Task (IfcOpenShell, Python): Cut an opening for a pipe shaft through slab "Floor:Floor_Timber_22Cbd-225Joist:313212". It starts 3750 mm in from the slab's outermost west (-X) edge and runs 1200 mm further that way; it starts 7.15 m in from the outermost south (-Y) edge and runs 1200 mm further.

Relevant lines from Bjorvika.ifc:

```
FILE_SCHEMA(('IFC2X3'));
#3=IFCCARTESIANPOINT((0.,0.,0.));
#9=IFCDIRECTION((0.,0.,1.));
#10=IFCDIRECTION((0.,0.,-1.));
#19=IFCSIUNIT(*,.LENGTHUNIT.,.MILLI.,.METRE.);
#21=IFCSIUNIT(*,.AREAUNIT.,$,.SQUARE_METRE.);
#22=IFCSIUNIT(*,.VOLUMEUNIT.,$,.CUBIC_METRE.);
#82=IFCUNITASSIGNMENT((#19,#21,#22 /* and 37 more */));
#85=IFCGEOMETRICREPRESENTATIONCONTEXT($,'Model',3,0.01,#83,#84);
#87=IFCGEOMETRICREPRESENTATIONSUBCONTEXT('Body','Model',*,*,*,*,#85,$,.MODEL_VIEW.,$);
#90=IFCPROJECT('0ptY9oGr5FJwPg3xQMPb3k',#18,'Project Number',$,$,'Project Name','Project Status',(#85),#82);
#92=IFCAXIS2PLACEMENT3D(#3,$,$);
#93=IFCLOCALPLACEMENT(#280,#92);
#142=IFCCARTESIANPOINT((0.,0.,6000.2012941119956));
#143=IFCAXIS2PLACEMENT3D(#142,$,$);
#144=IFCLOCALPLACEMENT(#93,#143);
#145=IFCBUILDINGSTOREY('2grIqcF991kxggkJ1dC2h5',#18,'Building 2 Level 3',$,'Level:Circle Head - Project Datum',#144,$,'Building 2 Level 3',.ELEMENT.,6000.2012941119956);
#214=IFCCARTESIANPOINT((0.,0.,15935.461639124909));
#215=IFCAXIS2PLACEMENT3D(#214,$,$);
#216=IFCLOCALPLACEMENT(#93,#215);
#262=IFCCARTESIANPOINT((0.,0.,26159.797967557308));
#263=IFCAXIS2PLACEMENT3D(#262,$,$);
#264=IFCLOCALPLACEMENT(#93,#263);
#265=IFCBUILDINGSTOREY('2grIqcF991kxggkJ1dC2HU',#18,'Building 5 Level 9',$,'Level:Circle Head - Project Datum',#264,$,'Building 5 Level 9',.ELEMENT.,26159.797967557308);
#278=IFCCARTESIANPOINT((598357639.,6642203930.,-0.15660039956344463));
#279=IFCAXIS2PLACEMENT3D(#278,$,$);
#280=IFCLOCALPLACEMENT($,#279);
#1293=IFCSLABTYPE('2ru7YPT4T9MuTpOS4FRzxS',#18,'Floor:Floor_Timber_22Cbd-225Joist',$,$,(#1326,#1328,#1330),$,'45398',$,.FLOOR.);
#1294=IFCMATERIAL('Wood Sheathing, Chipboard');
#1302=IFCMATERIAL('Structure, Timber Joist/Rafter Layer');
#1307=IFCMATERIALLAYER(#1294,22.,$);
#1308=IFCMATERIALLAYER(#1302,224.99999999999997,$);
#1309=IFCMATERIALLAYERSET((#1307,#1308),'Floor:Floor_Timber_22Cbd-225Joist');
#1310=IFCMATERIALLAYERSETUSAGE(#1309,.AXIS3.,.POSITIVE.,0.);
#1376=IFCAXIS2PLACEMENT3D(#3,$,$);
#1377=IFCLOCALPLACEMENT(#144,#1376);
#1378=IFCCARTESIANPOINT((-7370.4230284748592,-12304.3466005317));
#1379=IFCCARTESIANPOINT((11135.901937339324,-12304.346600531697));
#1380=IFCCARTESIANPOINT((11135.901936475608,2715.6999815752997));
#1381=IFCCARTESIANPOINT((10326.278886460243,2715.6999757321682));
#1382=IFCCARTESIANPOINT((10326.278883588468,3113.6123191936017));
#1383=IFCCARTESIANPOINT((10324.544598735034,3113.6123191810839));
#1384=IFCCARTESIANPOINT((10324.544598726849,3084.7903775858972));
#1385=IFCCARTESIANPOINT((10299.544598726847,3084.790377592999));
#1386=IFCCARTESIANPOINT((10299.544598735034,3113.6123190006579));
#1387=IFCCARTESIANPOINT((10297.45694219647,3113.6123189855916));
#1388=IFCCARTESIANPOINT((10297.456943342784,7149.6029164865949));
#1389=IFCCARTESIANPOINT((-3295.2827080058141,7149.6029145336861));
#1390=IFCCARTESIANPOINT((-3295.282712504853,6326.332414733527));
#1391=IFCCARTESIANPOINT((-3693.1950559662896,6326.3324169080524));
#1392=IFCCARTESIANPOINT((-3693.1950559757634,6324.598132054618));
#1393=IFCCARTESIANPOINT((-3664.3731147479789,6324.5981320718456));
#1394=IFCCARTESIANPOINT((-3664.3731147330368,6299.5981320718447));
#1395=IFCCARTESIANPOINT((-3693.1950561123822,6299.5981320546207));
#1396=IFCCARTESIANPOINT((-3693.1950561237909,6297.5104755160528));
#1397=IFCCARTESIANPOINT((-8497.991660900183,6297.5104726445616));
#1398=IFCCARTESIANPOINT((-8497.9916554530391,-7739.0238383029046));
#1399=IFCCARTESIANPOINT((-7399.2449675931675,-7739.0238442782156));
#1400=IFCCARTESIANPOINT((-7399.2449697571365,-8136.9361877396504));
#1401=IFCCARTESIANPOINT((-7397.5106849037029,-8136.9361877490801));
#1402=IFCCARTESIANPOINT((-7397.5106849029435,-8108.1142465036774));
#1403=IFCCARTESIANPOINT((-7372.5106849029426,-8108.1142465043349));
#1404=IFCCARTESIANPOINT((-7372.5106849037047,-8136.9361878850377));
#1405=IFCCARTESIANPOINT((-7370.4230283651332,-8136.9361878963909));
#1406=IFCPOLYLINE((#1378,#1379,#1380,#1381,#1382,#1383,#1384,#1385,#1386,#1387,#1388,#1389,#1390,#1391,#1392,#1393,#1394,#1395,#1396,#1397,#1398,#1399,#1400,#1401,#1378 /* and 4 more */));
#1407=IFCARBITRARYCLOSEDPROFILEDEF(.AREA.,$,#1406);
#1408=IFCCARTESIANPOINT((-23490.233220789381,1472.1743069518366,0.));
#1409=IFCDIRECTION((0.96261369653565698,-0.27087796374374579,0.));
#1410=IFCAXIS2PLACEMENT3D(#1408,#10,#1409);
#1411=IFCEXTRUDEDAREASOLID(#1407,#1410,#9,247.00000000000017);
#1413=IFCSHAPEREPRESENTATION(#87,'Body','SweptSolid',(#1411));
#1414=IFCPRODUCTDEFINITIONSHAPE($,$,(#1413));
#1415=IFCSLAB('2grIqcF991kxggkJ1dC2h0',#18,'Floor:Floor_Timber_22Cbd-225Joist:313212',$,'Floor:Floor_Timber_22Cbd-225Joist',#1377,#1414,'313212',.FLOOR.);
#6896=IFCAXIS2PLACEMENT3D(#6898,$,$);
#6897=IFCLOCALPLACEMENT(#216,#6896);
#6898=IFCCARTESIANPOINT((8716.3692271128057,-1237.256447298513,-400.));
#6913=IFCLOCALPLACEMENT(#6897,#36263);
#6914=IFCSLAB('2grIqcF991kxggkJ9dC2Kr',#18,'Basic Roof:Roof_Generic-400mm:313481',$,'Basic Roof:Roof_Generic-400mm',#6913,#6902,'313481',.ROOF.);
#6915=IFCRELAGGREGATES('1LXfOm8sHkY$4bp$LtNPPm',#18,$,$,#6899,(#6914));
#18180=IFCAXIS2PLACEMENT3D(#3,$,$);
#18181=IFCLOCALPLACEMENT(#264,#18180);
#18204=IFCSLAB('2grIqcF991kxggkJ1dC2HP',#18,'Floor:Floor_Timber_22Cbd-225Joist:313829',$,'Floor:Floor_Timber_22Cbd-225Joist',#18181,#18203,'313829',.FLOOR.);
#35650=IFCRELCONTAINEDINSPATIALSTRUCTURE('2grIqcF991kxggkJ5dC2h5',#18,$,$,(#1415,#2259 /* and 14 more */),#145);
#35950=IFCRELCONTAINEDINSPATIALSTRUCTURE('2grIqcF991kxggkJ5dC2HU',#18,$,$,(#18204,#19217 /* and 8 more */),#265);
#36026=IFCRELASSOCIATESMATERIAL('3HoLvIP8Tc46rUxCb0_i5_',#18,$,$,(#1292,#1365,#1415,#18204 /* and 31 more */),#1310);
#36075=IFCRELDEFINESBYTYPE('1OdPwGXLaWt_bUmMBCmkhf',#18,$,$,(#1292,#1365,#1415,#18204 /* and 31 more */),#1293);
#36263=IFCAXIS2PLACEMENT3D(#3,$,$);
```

```python
import numpy as np
import ifcopenshell
import ifcopenshell.api.feature
import ifcopenshell.api.geometry
import ifcopenshell.api.root
import ifcopenshell.geom
import ifcopenshell.util.placement
import ifcopenshell.util.representation
import ifcopenshell.util.shape
import ifcopenshell.util.unit

model = ifcopenshell.open("Bjorvika.ifc")
unit_scale = ifcopenshell.util.unit.calculate_unit_scale(model)
settings = ifcopenshell.geom.settings()


def volume(element):
    """Net volume in cubic metres, openings subtracted."""
    shape = ifcopenshell.geom.create_shape(settings, element)
    return ifcopenshell.util.shape.get_volume(shape.geometry)


slab = model.by_id(1415)
before = volume(slab)

# Extent in the slab's own axes, in metres. The edges named are its -X and -Y sides.
slab_shape = ifcopenshell.geom.create_shape(settings, slab)
vertices = ifcopenshell.util.shape.get_vertices(slab_shape.geometry)
x_min, y_min, bottom = vertices.min(axis=0)
top = vertices[:, 2].max()

opening = ifcopenshell.api.root.create_entity(model, ifc_class="IfcOpeningElement", name="Pipe shaft opening")
context = ifcopenshell.util.representation.get_context(model, "Model", "Body", "MODEL_VIEW")
width, depth = 1.2, 1.2
outline = [(0.0, 0.0), (width, 0.0), (width, depth), (0.0, depth), (0.0, 0.0)]
# Overshoot both faces by 50 mm so the cut is clean.
shape = ifcopenshell.api.geometry.add_slab_representation(
    model, context=context, depth=top - bottom + 0.1, polyline=outline
)
ifcopenshell.api.geometry.assign_representation(model, product=opening, representation=shape)

matrix = ifcopenshell.util.placement.get_local_placement(slab.ObjectPlacement)
matrix[:, 3] = matrix @ np.append(np.array([x_min + 3.75, y_min + 7.15, bottom - 0.05]) / unit_scale, 1.0)
ifcopenshell.api.geometry.edit_object_placement(model, product=opening, matrix=matrix, is_si=False)
ifcopenshell.api.feature.add_feature(model, feature=opening, element=slab)

after = volume(slab)

print(f"slab volume {before:.3f} -> {after:.3f} m3")

model.write("Bjorvika-out.ifc")
```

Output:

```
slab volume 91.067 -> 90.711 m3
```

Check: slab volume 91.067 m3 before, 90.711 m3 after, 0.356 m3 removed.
